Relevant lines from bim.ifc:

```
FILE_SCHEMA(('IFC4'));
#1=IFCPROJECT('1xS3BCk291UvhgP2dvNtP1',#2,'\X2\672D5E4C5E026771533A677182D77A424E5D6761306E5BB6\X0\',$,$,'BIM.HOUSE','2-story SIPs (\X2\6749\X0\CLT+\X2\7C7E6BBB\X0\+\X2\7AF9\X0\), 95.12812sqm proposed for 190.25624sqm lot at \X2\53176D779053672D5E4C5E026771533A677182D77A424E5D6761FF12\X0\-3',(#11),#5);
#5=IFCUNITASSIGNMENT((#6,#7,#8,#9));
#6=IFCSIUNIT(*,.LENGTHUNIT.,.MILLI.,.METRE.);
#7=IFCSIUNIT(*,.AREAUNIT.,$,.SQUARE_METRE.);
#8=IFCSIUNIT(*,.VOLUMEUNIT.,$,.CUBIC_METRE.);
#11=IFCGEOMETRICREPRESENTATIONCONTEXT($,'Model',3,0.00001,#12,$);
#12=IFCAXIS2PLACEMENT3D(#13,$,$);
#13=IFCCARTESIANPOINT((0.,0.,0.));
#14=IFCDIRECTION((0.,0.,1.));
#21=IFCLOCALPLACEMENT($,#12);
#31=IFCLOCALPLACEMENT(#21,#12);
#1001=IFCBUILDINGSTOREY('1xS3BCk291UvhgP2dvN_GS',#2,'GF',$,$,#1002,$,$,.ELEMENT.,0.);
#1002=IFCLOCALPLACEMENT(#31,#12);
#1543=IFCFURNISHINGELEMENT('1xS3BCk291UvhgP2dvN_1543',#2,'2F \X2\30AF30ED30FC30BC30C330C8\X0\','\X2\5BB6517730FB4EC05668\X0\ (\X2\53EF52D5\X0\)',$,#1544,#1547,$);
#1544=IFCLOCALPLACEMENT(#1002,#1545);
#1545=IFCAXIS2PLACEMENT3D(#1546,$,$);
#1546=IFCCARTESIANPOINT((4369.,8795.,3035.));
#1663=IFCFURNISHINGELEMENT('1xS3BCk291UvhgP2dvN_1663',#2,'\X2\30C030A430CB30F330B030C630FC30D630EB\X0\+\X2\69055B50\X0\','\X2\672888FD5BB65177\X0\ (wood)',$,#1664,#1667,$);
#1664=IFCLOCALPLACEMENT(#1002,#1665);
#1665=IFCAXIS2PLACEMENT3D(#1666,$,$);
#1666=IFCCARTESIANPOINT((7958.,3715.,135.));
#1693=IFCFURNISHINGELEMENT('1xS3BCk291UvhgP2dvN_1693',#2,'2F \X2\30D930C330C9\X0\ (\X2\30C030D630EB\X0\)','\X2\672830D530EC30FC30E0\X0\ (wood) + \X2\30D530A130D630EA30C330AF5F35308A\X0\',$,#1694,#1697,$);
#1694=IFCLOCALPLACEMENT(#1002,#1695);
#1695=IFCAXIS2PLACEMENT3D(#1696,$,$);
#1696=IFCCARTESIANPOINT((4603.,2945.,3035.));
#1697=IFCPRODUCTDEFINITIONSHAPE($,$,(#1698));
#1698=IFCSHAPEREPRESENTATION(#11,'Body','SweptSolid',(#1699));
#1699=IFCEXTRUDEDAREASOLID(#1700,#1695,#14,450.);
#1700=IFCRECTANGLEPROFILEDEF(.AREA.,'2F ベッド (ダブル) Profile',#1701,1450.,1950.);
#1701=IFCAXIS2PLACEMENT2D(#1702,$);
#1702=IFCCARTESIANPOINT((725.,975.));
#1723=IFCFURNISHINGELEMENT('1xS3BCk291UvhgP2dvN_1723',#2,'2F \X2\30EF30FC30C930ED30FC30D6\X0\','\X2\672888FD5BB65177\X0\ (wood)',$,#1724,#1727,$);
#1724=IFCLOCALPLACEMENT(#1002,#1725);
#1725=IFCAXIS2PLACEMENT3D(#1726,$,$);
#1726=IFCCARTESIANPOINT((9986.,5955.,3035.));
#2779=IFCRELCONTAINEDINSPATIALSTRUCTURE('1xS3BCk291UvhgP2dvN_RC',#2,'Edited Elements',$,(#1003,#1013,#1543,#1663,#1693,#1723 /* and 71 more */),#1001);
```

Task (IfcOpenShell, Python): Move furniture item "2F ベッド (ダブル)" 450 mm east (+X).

```python
import ifcopenshell
import ifcopenshell.api.geometry
import ifcopenshell.util.placement

model = ifcopenshell.open("bim.ifc")

item = model.by_guid("1xS3BCk291UvhgP2dvN_1693")
matrix = ifcopenshell.util.placement.get_local_placement(item.ObjectPlacement)
matrix[0, 3] += 450.0
ifcopenshell.api.geometry.edit_object_placement(model, product=item, matrix=matrix, is_si=False)

print(ifcopenshell.util.placement.get_local_placement(item.ObjectPlacement).round(3) + 0.0)

model.write("bim_edited.ifc")
```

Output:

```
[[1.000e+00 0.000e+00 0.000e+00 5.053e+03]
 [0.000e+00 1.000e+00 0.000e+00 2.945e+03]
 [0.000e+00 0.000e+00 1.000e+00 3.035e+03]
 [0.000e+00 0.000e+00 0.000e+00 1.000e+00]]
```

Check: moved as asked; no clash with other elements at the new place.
